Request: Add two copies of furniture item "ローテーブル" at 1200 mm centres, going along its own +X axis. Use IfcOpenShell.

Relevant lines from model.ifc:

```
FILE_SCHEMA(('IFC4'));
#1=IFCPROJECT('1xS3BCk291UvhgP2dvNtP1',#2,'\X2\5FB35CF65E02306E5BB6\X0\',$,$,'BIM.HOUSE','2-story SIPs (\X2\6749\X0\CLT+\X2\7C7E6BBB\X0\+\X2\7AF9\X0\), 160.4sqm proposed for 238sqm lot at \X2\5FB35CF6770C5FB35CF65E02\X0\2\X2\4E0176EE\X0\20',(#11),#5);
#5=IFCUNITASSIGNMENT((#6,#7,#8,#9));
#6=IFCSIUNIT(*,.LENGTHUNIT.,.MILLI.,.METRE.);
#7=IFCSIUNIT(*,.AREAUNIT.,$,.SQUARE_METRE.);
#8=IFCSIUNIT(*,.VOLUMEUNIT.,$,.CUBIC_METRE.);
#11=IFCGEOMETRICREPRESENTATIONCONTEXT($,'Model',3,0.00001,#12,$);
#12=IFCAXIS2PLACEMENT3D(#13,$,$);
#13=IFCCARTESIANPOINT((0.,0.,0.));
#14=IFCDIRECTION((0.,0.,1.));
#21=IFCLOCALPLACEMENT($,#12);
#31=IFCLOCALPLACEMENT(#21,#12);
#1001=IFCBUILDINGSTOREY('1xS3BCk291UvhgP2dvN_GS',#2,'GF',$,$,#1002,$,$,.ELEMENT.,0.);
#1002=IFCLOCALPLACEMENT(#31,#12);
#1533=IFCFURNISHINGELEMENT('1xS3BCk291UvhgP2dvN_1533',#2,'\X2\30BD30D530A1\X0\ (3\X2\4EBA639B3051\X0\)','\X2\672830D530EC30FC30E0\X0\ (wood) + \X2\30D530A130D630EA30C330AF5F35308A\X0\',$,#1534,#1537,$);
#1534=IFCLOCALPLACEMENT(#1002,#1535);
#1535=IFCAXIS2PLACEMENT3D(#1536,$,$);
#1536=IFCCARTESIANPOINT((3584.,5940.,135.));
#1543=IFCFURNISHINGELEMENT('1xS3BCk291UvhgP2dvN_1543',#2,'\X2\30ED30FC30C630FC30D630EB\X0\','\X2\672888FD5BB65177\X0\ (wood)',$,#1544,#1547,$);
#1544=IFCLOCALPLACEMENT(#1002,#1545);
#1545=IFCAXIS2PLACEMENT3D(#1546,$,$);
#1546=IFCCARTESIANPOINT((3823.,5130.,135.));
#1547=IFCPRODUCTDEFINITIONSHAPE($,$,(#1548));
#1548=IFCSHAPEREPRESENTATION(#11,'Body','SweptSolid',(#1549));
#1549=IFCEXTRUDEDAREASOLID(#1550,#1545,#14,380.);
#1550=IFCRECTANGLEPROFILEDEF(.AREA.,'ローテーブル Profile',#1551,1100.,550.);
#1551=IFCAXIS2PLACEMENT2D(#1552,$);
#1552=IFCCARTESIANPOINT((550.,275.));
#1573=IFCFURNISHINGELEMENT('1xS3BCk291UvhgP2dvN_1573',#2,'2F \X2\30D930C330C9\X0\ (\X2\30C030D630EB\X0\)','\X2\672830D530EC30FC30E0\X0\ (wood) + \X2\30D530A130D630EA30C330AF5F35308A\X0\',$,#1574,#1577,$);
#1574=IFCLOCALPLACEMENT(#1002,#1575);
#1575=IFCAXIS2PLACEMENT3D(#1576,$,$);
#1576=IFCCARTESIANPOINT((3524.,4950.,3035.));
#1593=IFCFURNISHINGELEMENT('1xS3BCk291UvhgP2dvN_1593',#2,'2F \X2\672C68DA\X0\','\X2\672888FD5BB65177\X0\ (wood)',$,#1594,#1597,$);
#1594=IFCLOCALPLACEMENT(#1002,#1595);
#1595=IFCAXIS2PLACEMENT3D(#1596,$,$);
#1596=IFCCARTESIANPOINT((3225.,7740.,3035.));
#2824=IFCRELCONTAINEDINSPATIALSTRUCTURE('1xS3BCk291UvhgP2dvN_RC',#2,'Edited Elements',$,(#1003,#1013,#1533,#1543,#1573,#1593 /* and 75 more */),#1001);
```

```python
import ifcopenshell
import ifcopenshell.api.geometry
import ifcopenshell.api.root
import ifcopenshell.util.element
import ifcopenshell.util.placement

model = ifcopenshell.open("model.ifc")


def reuse_history(source, copy):
    """copy_class also copies each property set's owner history, people and application; keep the originals."""
    for rel in copy.IsDefinedBy:
        if rel.is_a("IfcRelDefinesByProperties") and (history := rel.RelatingPropertyDefinition.OwnerHistory):
            rel.RelatingPropertyDefinition.OwnerHistory = source.OwnerHistory
            ifcopenshell.util.element.remove_deep2(model, history)


source = model.by_guid("1xS3BCk291UvhgP2dvN_1543")
base = ifcopenshell.util.placement.get_local_placement(source.ObjectPlacement)
step = base[:3, 0] * 1200.0

for i in range(1, 3):
    copy = ifcopenshell.api.root.copy_class(model, product=source)
    copy.Representation = ifcopenshell.util.element.copy_deep(
        model, source.Representation, exclude=["IfcGeometricRepresentationContext", "IfcRepresentationMap"]
    )
    reuse_history(source, copy)
    matrix = base.copy()
    matrix[:3, 3] += i * step
    print("added at", matrix[:3, 3].round(3) + 0.0)
    ifcopenshell.api.geometry.edit_object_placement(model, product=copy, matrix=matrix, is_si=False)

model.write("model_v2.ifc")
```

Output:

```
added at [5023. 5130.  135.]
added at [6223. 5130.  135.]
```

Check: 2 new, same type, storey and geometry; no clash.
